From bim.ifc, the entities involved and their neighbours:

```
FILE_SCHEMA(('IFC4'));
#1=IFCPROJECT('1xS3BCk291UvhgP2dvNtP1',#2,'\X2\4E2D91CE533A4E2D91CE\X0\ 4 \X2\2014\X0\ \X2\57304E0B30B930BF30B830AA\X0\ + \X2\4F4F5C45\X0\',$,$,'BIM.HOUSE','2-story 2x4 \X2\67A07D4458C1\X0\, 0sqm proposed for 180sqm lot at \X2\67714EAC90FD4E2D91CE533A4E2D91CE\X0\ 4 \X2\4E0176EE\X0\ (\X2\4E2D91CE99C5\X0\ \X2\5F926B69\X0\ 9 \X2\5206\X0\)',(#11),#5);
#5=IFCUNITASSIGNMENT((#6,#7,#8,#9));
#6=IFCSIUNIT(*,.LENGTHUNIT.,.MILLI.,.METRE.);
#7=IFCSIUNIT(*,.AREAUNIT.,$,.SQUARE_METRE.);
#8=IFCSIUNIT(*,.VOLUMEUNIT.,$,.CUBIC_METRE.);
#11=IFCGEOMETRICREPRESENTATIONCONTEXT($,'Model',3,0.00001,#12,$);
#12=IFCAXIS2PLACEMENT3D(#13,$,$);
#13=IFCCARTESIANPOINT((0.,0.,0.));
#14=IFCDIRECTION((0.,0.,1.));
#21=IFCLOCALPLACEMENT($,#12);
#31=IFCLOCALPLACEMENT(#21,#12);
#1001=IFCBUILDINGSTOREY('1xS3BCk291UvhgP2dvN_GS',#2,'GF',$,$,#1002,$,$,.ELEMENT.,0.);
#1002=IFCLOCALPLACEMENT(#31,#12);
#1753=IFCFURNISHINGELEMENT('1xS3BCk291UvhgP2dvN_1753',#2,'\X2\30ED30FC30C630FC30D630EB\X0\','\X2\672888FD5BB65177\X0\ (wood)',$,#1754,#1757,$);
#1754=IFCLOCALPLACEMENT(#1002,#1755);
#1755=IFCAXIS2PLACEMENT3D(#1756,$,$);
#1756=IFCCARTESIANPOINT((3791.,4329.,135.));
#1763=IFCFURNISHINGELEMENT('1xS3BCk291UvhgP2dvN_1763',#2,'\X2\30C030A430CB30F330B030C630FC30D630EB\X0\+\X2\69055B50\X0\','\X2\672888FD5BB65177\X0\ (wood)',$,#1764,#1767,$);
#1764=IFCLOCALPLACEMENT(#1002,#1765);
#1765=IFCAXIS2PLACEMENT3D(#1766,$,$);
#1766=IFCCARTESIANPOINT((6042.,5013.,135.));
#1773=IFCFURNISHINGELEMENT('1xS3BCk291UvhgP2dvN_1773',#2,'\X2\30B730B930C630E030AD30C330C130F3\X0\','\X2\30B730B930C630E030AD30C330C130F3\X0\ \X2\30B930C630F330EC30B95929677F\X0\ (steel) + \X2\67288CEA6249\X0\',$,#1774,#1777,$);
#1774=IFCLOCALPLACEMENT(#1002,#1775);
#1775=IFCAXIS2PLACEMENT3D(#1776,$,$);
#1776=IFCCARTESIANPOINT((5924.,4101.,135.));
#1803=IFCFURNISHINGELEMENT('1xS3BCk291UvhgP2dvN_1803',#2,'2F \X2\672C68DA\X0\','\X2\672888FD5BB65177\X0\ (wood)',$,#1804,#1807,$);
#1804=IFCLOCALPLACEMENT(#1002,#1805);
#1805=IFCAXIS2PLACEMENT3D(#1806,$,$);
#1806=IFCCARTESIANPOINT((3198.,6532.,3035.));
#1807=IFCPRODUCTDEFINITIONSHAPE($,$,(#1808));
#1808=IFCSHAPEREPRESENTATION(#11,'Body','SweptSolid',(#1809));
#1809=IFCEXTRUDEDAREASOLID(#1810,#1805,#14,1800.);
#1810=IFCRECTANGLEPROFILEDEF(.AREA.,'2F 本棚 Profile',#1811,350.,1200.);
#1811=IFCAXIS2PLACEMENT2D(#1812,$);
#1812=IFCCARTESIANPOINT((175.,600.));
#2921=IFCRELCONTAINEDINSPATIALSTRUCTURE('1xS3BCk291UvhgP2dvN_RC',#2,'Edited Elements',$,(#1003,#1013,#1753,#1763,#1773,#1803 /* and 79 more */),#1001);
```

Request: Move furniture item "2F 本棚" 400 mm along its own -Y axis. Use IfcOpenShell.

```python
import ifcopenshell
import ifcopenshell.api.geometry
import ifcopenshell.util.placement

model = ifcopenshell.open("bim.ifc")

item = model.by_id(1803)
matrix = ifcopenshell.util.placement.get_local_placement(item.ObjectPlacement)
matrix[:3, 3] -= matrix[:3, 1] * 400.0
ifcopenshell.api.geometry.edit_object_placement(model, product=item, matrix=matrix, is_si=False)

print(ifcopenshell.util.placement.get_local_placement(item.ObjectPlacement).round(3) + 0.0)

model.write("bim_updated.ifc")
```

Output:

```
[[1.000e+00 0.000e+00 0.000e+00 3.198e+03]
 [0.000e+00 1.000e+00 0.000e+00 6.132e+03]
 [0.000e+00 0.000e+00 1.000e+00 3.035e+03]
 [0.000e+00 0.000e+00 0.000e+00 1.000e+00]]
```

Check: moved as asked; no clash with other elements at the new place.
